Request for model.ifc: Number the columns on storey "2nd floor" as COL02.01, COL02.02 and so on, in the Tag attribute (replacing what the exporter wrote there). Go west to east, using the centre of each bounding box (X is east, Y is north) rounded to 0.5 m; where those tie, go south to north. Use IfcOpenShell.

First a look at what the model holds.

```python
import ifcopenshell
import ifcopenshell.util.element
import ifcopenshell.util.placement

model = ifcopenshell.open("model.ifc")
print(model.schema)
storey = next(s for s in model.by_type("IfcBuildingStorey") if s.Name == "2nd floor")
columns = [e for e in ifcopenshell.util.element.get_decomposition(storey) if e.is_a("IfcColumn")]
for e in sorted(columns, key=lambda e: e.id()):
    origin = ifcopenshell.util.placement.get_local_placement(e.ObjectPlacement)[:3, 3]
    print(e.id(), e.Tag, e.Name, origin.round(2) + 0.0, sep=" | ")
```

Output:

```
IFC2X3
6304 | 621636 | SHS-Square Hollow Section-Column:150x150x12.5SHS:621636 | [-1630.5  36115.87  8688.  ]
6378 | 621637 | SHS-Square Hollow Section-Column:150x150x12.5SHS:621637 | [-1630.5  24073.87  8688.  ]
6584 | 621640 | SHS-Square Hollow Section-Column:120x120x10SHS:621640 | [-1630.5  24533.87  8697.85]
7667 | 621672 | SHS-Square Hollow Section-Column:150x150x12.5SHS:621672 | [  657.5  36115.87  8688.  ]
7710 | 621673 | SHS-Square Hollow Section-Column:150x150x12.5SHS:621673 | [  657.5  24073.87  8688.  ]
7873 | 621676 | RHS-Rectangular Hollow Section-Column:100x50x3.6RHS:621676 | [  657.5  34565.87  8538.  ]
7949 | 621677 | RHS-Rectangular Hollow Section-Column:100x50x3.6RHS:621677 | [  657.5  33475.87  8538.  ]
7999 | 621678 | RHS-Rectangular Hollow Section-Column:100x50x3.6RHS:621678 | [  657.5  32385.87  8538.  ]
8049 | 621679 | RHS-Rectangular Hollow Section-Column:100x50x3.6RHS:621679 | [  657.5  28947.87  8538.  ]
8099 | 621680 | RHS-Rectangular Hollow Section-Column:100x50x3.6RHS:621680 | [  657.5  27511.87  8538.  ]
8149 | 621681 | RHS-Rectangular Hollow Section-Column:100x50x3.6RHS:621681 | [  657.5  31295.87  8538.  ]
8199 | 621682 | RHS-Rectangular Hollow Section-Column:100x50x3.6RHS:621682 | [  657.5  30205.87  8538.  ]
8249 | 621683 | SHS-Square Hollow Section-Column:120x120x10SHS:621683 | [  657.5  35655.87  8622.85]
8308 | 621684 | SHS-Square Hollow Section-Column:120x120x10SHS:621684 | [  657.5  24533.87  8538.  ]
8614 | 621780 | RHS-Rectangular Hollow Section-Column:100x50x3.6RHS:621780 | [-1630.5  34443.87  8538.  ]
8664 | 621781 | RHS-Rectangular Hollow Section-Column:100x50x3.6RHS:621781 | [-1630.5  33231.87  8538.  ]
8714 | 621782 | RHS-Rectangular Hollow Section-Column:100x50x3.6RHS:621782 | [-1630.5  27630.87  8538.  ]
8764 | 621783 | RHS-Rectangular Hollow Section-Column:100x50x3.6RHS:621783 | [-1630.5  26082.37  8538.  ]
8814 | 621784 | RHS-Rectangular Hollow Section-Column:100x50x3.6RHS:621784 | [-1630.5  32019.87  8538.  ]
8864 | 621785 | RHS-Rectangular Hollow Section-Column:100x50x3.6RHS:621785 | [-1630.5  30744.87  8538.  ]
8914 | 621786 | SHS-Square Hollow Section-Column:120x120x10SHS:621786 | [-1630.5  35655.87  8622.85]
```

```python
import ifcopenshell
import ifcopenshell.geom
import ifcopenshell.util.element
import ifcopenshell.util.shape

model = ifcopenshell.open("model.ifc")
settings = ifcopenshell.geom.settings()
settings.set("use-world-coords", True)


def centre(element):
    shape = ifcopenshell.geom.create_shape(settings, element)
    return ifcopenshell.util.shape.get_bbox_centroid(shape.geometry)


storey = next(s for s in model.by_type("IfcBuildingStorey") if s.Name == "2nd floor")
columns = [e for e in ifcopenshell.util.element.get_decomposition(storey) if e.is_a("IfcColumn")]

# Insertion points can sit at a corner or the storey origin, so sort by the geometry (in metres).
centres = {e: centre(e) for e in columns}
columns.sort(key=lambda e: (round(centres[e][0] / 0.5), centres[e][1]))

for i, e in enumerate(columns, start=1):
    number = f"COL02.{i:02d}"
    e.Tag = number
    print(e.id(), number)

model.write("model_rev.ifc")
```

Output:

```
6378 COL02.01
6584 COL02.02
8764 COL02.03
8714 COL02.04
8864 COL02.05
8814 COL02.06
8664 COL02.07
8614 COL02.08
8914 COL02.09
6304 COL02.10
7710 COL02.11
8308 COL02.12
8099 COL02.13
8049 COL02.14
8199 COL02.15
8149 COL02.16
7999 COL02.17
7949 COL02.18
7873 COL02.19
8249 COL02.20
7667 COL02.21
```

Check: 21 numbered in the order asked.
